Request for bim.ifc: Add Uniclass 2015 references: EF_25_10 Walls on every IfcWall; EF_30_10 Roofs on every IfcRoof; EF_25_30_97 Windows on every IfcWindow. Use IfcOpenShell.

First a look at what the model holds.

```python
import ifcopenshell

model = ifcopenshell.open("bim.ifc")
print(model.schema)
print("classifications:", [c.Name for c in model.by_type("IfcClassification")])
for ifc_class in ("IfcDoor", "IfcRoof", "IfcStair", "IfcWall", "IfcWindow"):
    print(ifc_class, len(model.by_type(ifc_class)))
```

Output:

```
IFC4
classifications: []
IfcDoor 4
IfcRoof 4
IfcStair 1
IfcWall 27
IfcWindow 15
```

```python
import ifcopenshell
import ifcopenshell.api.classification

model = ifcopenshell.open("bim.ifc")

system = ifcopenshell.api.classification.add_classification(model, classification="Uniclass 2015")

codes = {
    "IfcWall": ("EF_25_10", "Walls"),
    "IfcRoof": ("EF_30_10", "Roofs"),
    "IfcWindow": ("EF_25_30_97", "Windows"),
}
for ifc_class, (code, name) in codes.items():
    products = model.by_type(ifc_class)
    ifcopenshell.api.classification.add_reference(
        model, products=products, classification=system, identification=code, name=name
    )
    print(code, len(products))

model.write("bim_edited.ifc")
```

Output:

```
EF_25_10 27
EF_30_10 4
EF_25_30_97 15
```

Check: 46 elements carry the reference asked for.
